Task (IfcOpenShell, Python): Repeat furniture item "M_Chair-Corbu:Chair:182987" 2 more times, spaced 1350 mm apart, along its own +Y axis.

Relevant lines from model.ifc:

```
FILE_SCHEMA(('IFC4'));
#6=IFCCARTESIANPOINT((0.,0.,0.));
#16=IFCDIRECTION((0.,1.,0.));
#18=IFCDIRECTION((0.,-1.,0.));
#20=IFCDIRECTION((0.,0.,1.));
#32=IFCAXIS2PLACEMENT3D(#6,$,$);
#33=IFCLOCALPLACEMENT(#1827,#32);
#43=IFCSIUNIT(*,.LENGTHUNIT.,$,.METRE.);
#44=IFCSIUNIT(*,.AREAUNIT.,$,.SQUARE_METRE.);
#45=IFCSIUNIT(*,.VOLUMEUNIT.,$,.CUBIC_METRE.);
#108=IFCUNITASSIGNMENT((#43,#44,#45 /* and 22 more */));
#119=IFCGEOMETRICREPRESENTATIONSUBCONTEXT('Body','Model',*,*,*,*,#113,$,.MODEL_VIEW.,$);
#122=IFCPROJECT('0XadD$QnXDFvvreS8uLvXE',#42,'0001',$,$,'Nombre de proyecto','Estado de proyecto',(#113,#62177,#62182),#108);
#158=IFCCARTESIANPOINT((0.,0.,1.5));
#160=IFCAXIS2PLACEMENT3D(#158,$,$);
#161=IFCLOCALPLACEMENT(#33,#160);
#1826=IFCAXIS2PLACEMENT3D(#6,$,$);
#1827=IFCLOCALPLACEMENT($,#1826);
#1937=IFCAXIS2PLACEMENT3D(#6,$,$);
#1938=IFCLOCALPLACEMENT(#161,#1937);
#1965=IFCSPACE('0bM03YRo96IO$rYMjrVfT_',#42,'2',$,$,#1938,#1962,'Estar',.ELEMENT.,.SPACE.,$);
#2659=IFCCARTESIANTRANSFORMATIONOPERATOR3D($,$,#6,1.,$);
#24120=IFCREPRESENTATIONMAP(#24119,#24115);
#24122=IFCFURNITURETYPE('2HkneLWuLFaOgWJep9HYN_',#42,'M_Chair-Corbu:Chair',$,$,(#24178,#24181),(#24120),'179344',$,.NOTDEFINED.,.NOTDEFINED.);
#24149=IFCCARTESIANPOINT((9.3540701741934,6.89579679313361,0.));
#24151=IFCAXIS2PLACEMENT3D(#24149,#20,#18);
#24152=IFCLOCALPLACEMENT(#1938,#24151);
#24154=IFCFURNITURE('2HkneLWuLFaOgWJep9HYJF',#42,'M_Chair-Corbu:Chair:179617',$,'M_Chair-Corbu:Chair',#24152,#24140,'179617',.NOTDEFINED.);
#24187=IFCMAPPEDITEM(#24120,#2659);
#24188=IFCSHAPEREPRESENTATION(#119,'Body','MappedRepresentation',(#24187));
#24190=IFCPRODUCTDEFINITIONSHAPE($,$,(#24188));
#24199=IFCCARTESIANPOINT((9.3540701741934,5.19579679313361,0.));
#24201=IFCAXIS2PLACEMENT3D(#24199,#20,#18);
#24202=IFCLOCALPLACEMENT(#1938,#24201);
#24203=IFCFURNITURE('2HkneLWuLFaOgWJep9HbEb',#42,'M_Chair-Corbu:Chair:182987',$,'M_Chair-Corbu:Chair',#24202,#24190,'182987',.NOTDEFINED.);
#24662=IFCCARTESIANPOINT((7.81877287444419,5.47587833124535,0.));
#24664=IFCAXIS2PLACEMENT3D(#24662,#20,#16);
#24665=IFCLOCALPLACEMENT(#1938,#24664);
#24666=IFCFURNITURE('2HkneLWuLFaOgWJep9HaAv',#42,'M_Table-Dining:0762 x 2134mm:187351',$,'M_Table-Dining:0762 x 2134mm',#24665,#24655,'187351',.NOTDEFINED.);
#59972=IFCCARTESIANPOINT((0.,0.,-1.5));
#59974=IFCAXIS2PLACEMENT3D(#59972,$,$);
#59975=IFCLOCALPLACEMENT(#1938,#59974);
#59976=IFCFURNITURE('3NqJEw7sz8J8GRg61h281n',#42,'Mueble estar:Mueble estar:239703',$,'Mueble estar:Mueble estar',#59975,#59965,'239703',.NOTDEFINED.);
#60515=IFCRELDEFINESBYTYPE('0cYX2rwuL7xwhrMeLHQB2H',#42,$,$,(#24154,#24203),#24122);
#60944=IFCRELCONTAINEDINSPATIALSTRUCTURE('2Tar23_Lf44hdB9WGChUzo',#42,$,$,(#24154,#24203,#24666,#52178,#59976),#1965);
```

```python
import ifcopenshell
import ifcopenshell.api.geometry
import ifcopenshell.api.root
import ifcopenshell.util.element
import ifcopenshell.util.placement

model = ifcopenshell.open("model.ifc")


def reuse_history(source, copy):
    """copy_class also copies each property set's owner history, people and application; keep the originals."""
    for rel in copy.IsDefinedBy:
        if rel.is_a("IfcRelDefinesByProperties") and (history := rel.RelatingPropertyDefinition.OwnerHistory):
            rel.RelatingPropertyDefinition.OwnerHistory = source.OwnerHistory
            ifcopenshell.util.element.remove_deep2(model, history)


source = model.by_id(24203)
base = ifcopenshell.util.placement.get_local_placement(source.ObjectPlacement)
step = base[:3, 1] * 1.35

for i in range(1, 3):
    copy = ifcopenshell.api.root.copy_class(model, product=source)
    copy.Representation = ifcopenshell.util.element.copy_deep(
        model, source.Representation, exclude=["IfcGeometricRepresentationContext", "IfcRepresentationMap"]
    )
    copy.Name = "M_Chair-Corbu:Chair"
    copy.Tag = None
    reuse_history(source, copy)
    matrix = base.copy()
    matrix[:3, 3] += i * step
    print("added at", matrix[:3, 3].round(3) + 0.0)
    ifcopenshell.api.geometry.edit_object_placement(model, product=copy, matrix=matrix, is_si=False)

model.write("model-out.ifc")
```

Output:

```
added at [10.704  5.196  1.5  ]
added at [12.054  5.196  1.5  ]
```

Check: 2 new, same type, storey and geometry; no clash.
